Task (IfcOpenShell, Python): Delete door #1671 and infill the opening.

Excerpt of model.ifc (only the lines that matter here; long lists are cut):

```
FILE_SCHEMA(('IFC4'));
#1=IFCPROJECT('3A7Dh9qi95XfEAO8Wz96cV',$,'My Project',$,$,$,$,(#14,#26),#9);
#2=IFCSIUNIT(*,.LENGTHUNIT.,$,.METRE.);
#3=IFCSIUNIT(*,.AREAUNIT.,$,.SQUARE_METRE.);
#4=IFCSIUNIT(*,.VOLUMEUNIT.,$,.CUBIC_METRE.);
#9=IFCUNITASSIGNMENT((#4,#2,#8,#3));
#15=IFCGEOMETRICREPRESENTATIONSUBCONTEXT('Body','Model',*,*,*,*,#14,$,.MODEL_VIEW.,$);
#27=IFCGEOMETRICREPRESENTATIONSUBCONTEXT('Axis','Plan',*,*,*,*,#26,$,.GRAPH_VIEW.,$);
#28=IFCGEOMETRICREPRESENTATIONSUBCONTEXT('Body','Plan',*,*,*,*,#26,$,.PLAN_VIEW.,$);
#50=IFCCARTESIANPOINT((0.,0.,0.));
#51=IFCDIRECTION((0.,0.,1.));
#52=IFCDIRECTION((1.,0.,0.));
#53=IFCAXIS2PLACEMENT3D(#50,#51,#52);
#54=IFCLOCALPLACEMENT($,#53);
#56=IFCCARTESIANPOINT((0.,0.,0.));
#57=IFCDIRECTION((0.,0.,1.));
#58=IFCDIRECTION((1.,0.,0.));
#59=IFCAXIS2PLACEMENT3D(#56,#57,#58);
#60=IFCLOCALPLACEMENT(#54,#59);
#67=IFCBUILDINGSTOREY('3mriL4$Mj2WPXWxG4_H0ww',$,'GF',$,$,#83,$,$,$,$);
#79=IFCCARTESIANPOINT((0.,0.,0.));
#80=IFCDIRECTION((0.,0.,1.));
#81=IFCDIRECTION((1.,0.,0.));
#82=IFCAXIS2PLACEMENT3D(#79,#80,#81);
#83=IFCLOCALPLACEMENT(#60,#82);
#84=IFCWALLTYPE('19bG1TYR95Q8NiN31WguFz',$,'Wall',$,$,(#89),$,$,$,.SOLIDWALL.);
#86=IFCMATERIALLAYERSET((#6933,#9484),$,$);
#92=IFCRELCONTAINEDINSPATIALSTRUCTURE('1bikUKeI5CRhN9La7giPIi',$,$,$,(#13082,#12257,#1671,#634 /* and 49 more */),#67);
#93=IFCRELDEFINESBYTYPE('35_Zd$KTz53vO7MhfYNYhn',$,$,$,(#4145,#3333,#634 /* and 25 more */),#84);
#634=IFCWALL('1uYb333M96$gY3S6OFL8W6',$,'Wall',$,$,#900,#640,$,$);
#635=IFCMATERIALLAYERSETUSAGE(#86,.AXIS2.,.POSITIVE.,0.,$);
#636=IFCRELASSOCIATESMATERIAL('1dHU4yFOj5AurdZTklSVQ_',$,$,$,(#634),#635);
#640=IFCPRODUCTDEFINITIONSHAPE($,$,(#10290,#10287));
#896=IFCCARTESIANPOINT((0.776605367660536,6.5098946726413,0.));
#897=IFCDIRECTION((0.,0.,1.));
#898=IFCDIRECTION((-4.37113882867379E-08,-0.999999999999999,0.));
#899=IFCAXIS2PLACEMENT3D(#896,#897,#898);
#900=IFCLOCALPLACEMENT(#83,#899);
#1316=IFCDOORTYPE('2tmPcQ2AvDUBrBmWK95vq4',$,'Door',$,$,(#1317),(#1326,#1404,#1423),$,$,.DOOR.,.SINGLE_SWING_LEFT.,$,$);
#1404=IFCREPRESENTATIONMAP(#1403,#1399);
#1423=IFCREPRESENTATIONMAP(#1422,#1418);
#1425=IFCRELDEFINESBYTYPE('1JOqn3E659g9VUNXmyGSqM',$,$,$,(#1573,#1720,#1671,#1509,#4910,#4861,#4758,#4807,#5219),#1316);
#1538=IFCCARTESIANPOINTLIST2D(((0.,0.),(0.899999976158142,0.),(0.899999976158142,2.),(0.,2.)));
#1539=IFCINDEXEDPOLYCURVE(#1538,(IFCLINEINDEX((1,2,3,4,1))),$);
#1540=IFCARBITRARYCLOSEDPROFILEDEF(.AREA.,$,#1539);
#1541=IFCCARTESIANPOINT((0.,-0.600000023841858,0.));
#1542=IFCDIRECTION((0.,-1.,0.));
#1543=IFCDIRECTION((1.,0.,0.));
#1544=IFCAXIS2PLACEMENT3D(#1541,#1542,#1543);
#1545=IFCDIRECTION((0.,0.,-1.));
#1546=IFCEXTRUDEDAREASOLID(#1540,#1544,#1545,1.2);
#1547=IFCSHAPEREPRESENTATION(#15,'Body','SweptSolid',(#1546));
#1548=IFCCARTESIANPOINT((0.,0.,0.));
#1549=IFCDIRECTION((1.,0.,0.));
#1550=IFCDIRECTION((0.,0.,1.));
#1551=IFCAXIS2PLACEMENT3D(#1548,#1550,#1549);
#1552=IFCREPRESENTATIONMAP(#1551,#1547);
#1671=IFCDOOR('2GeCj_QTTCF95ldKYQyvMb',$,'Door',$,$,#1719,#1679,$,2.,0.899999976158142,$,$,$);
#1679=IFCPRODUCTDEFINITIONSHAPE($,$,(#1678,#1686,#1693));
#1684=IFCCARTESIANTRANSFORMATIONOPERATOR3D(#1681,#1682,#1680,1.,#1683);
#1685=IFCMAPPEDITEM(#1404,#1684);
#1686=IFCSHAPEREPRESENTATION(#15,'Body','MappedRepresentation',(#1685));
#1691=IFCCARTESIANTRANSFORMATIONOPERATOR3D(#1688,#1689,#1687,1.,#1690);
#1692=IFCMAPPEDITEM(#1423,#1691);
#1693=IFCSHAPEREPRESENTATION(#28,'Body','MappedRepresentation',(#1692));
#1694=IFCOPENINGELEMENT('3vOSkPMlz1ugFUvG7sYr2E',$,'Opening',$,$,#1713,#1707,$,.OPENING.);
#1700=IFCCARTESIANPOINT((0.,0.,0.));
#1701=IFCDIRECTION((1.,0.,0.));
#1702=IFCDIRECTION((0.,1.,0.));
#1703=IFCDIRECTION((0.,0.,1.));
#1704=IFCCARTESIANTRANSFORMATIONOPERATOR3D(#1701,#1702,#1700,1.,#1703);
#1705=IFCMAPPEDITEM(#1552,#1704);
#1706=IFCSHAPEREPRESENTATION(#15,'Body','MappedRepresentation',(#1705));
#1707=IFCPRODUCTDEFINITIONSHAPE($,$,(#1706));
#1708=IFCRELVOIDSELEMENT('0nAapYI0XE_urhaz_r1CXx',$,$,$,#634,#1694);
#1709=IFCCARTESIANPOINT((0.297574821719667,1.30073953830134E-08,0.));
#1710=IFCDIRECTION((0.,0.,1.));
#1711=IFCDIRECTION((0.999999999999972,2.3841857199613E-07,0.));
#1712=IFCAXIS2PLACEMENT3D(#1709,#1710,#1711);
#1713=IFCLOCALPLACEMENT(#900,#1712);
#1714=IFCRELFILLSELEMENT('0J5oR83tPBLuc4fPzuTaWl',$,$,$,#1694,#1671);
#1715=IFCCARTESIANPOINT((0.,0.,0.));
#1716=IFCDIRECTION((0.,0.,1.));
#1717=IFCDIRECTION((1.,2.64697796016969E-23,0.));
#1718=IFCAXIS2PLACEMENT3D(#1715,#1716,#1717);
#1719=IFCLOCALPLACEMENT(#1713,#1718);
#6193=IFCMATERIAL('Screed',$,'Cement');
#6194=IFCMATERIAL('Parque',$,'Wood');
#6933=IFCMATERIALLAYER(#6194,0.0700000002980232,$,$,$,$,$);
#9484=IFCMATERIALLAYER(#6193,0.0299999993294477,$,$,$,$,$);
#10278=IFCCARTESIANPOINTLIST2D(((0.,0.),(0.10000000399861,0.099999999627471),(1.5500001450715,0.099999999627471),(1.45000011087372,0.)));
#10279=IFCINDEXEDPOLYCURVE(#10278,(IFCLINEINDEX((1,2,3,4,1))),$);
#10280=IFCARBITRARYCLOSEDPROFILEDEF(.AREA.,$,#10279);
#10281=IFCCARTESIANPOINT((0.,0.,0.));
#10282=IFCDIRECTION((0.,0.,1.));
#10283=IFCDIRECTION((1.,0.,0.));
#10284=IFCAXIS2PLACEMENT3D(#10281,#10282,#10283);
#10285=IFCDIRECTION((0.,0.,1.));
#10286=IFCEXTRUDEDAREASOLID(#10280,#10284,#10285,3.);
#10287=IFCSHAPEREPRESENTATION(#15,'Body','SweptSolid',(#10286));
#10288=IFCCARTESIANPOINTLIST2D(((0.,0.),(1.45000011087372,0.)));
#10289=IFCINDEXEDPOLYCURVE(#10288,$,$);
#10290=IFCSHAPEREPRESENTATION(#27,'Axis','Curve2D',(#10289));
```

```python
import ifcopenshell
import ifcopenshell.api.feature
import ifcopenshell.api.root
import ifcopenshell.geom
import ifcopenshell.util.shape

model = ifcopenshell.open("model.ifc")
settings = ifcopenshell.geom.settings()


def volume(element):
    """Net volume in cubic metres, openings subtracted."""
    shape = ifcopenshell.geom.create_shape(settings, element)
    return ifcopenshell.util.shape.get_volume(shape.geometry)


door = model.by_id(1671)
opening = door.FillsVoids[0].RelatingOpeningElement
wall = opening.VoidsElements[0].RelatingBuildingElement
before = volume(wall)

ifcopenshell.api.root.remove_product(model, product=door)
ifcopenshell.api.feature.remove_feature(model, feature=opening)

after = volume(wall)

print(f"wall volume {before:.3f} -> {after:.3f} m3")

model.write("model-out.ifc")
```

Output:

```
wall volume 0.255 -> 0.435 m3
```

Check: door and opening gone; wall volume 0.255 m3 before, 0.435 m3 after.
